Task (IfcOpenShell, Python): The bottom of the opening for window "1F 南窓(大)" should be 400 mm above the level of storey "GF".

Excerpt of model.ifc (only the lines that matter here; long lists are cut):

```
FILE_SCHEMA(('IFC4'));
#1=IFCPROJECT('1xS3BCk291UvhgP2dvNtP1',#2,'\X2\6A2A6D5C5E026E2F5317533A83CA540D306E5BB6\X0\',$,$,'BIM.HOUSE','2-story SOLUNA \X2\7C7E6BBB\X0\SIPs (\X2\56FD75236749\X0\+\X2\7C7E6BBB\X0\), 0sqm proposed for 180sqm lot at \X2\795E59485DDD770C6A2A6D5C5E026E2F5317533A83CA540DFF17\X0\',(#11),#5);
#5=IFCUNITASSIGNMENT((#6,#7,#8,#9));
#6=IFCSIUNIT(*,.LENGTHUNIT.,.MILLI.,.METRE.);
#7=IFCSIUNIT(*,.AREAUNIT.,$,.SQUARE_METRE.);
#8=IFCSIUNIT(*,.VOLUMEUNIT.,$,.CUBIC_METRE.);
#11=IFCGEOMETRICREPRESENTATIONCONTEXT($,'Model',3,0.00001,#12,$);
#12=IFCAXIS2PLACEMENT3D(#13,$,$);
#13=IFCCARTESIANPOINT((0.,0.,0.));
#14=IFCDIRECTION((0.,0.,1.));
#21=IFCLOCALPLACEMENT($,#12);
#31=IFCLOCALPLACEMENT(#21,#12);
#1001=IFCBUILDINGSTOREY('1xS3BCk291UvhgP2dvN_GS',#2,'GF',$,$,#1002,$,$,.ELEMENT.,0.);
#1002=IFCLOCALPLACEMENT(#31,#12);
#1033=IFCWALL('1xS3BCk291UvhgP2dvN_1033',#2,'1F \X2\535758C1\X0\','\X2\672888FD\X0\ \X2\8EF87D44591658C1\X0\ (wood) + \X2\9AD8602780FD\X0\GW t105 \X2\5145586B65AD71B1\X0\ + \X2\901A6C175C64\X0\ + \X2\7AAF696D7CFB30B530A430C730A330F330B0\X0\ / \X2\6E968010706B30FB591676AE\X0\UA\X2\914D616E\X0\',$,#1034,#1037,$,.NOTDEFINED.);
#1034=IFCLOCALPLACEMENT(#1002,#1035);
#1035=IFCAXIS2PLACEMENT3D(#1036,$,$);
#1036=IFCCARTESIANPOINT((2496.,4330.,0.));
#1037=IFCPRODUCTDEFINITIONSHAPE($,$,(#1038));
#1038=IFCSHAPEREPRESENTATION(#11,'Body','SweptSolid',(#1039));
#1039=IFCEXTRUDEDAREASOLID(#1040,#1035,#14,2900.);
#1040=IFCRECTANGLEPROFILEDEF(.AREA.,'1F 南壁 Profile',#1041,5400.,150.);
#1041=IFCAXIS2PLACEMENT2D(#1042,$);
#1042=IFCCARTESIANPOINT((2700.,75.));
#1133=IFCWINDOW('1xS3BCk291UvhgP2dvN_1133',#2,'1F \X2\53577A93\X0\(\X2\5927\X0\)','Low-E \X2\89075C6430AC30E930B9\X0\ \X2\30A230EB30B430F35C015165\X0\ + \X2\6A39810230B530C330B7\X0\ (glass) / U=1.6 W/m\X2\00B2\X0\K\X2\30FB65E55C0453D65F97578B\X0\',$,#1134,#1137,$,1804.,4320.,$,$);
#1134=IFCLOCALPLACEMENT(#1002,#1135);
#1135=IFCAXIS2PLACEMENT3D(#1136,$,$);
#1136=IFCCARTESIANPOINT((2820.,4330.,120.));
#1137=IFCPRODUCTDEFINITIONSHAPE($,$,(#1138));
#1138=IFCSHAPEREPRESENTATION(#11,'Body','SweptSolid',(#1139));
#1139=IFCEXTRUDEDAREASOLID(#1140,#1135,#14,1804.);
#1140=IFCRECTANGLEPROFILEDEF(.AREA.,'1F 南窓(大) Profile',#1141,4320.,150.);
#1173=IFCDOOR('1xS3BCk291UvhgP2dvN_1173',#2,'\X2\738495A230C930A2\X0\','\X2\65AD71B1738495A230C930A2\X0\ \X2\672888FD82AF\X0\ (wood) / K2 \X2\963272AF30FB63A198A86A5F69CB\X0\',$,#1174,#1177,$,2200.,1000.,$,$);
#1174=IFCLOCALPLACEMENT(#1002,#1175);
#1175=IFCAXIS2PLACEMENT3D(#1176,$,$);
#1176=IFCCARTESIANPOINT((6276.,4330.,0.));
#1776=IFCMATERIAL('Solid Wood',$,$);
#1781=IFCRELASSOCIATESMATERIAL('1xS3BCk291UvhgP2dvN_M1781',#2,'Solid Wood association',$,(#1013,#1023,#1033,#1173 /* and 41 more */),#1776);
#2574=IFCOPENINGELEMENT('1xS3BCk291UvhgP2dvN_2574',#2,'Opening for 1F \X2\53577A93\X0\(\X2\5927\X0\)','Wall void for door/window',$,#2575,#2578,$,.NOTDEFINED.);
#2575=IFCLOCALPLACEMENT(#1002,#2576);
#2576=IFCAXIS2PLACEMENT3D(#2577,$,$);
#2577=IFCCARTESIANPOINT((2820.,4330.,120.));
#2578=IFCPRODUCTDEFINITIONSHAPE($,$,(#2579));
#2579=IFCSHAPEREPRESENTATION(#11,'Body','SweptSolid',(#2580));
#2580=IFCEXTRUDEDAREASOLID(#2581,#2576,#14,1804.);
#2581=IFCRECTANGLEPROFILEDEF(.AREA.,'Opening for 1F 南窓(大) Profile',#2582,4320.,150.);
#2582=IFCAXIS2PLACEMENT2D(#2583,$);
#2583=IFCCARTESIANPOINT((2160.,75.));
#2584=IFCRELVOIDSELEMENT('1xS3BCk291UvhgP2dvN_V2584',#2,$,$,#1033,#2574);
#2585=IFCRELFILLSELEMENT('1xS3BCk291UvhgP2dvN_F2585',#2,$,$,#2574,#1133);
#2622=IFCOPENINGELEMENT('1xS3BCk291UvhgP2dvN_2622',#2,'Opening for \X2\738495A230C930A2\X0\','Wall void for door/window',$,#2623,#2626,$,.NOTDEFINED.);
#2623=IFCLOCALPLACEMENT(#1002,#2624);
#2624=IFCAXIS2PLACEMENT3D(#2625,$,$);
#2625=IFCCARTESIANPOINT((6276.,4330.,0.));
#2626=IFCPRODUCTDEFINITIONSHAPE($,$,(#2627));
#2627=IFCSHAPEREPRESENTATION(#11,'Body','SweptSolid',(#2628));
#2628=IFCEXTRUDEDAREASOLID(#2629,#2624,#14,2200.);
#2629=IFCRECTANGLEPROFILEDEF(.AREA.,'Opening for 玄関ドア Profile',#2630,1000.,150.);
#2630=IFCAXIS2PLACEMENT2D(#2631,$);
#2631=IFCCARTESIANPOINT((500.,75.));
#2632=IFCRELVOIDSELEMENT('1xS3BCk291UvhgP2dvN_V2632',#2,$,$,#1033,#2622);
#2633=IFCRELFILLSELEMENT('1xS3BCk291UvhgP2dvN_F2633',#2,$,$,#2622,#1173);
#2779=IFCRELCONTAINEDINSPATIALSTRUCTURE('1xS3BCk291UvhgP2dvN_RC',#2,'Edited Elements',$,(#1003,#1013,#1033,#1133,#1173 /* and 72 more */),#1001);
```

```python
import numpy as np
import ifcopenshell
import ifcopenshell.api.geometry
import ifcopenshell.geom
import ifcopenshell.util.element
import ifcopenshell.util.placement
import ifcopenshell.util.shape
import ifcopenshell.util.unit

model = ifcopenshell.open("model.ifc")
unit_scale = ifcopenshell.util.unit.calculate_unit_scale(model)

window = model.by_guid("1xS3BCk291UvhgP2dvN_1133")
opening = window.FillsVoids[0].RelatingOpeningElement
storey = ifcopenshell.util.element.get_container(window, ifc_class="IfcBuildingStorey")
level = ifcopenshell.util.placement.get_local_placement(storey.ObjectPlacement)[2, 3]

# The opening's origin need not be at the sill, so measure its lowest point.
shape = ifcopenshell.geom.create_shape(ifcopenshell.geom.settings(), opening)
bottom = ifcopenshell.util.shape.get_shape_bottom_elevation(shape, shape.geometry) / unit_scale
dz = level + 0.4 / unit_scale - bottom

shift = np.array([0.0, 0.0, dz])
# The window is not placed relative to its opening, so move both.
for product in (opening, window):
    matrix = ifcopenshell.util.placement.get_local_placement(product.ObjectPlacement)
    matrix[:3, 3] += shift
    ifcopenshell.api.geometry.edit_object_placement(model, product=product, matrix=matrix, is_si=False)

print(f"moved by {dz * unit_scale:+.3f} m")

model.write("model_rev.ifc")
```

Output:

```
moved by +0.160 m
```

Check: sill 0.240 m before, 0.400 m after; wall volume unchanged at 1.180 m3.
